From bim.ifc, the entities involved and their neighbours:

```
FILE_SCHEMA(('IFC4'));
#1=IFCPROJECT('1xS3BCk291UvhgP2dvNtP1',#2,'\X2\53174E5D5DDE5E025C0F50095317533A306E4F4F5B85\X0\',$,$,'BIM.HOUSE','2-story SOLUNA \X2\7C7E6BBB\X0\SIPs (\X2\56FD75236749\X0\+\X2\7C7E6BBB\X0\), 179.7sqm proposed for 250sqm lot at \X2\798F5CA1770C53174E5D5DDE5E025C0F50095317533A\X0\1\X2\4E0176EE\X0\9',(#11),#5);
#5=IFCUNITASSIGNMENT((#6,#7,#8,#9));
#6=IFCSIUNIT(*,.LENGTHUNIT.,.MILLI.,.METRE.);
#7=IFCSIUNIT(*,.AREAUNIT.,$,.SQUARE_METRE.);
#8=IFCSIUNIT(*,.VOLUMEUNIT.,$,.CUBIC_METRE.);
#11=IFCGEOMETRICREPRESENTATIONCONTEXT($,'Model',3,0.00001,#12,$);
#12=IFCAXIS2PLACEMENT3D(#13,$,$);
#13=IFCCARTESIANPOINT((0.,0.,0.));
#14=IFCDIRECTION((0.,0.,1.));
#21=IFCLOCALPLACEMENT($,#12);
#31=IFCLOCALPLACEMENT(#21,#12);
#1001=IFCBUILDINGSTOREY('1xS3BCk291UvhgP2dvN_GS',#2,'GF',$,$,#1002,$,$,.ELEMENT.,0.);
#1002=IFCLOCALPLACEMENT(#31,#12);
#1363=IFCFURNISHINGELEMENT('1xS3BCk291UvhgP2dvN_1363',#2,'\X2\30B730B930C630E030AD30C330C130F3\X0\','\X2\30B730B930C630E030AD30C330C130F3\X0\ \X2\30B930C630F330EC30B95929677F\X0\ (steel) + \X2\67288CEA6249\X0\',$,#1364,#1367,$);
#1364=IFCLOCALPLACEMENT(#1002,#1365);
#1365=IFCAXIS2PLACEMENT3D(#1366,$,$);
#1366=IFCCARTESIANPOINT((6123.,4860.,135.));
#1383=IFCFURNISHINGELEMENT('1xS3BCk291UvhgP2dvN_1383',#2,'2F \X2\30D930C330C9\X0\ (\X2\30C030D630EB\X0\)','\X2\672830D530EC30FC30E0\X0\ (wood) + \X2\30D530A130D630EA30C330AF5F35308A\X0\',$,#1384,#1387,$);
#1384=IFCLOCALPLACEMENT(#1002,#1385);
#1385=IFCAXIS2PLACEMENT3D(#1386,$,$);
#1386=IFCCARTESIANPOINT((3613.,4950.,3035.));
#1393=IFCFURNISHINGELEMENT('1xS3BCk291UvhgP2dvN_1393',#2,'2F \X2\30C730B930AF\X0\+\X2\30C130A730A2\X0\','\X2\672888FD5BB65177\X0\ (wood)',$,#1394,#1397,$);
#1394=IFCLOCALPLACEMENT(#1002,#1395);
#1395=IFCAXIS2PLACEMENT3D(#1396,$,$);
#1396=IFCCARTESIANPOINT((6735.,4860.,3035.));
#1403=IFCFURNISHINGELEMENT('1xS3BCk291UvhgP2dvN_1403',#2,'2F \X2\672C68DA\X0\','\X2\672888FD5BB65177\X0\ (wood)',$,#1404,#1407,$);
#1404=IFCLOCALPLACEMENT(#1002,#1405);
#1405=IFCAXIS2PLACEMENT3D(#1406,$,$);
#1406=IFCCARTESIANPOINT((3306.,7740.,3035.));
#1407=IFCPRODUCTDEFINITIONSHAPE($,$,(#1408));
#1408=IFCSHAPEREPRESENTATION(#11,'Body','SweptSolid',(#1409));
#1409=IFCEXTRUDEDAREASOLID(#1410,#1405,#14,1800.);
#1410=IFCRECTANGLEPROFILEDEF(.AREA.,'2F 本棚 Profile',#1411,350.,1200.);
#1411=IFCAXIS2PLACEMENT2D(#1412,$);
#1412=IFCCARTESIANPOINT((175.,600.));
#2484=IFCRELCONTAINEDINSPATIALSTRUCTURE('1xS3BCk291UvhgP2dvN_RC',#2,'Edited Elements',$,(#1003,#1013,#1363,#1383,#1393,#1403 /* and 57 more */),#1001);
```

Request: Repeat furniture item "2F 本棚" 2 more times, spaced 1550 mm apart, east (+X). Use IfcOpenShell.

```python
import numpy as np
import ifcopenshell
import ifcopenshell.api.geometry
import ifcopenshell.api.root
import ifcopenshell.util.element
import ifcopenshell.util.placement
import ifcopenshell.util.unit

model = ifcopenshell.open("bim.ifc")
unit_scale = ifcopenshell.util.unit.calculate_unit_scale(model)


def reuse_history(source, copy):
    """copy_class also copies each property set's owner history, people and application; keep the originals."""
    for rel in copy.IsDefinedBy:
        if rel.is_a("IfcRelDefinesByProperties") and (history := rel.RelatingPropertyDefinition.OwnerHistory):
            rel.RelatingPropertyDefinition.OwnerHistory = source.OwnerHistory
            ifcopenshell.util.element.remove_deep2(model, history)


source = model.by_id(1403)
base = ifcopenshell.util.placement.get_local_placement(source.ObjectPlacement)
step = np.array([1.0, 0.0, 0.0]) * 1.55 / unit_scale

for i in range(1, 3):
    copy = ifcopenshell.api.root.copy_class(model, product=source)
    copy.Representation = ifcopenshell.util.element.copy_deep(
        model, source.Representation, exclude=["IfcGeometricRepresentationContext", "IfcRepresentationMap"]
    )
    reuse_history(source, copy)
    matrix = base.copy()
    matrix[:3, 3] += i * step
    print("added at", matrix[:3, 3].round(3) + 0.0)
    ifcopenshell.api.geometry.edit_object_placement(model, product=copy, matrix=matrix, is_si=False)

model.write("bim_v2.ifc")
```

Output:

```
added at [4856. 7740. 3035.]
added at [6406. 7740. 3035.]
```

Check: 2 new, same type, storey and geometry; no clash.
